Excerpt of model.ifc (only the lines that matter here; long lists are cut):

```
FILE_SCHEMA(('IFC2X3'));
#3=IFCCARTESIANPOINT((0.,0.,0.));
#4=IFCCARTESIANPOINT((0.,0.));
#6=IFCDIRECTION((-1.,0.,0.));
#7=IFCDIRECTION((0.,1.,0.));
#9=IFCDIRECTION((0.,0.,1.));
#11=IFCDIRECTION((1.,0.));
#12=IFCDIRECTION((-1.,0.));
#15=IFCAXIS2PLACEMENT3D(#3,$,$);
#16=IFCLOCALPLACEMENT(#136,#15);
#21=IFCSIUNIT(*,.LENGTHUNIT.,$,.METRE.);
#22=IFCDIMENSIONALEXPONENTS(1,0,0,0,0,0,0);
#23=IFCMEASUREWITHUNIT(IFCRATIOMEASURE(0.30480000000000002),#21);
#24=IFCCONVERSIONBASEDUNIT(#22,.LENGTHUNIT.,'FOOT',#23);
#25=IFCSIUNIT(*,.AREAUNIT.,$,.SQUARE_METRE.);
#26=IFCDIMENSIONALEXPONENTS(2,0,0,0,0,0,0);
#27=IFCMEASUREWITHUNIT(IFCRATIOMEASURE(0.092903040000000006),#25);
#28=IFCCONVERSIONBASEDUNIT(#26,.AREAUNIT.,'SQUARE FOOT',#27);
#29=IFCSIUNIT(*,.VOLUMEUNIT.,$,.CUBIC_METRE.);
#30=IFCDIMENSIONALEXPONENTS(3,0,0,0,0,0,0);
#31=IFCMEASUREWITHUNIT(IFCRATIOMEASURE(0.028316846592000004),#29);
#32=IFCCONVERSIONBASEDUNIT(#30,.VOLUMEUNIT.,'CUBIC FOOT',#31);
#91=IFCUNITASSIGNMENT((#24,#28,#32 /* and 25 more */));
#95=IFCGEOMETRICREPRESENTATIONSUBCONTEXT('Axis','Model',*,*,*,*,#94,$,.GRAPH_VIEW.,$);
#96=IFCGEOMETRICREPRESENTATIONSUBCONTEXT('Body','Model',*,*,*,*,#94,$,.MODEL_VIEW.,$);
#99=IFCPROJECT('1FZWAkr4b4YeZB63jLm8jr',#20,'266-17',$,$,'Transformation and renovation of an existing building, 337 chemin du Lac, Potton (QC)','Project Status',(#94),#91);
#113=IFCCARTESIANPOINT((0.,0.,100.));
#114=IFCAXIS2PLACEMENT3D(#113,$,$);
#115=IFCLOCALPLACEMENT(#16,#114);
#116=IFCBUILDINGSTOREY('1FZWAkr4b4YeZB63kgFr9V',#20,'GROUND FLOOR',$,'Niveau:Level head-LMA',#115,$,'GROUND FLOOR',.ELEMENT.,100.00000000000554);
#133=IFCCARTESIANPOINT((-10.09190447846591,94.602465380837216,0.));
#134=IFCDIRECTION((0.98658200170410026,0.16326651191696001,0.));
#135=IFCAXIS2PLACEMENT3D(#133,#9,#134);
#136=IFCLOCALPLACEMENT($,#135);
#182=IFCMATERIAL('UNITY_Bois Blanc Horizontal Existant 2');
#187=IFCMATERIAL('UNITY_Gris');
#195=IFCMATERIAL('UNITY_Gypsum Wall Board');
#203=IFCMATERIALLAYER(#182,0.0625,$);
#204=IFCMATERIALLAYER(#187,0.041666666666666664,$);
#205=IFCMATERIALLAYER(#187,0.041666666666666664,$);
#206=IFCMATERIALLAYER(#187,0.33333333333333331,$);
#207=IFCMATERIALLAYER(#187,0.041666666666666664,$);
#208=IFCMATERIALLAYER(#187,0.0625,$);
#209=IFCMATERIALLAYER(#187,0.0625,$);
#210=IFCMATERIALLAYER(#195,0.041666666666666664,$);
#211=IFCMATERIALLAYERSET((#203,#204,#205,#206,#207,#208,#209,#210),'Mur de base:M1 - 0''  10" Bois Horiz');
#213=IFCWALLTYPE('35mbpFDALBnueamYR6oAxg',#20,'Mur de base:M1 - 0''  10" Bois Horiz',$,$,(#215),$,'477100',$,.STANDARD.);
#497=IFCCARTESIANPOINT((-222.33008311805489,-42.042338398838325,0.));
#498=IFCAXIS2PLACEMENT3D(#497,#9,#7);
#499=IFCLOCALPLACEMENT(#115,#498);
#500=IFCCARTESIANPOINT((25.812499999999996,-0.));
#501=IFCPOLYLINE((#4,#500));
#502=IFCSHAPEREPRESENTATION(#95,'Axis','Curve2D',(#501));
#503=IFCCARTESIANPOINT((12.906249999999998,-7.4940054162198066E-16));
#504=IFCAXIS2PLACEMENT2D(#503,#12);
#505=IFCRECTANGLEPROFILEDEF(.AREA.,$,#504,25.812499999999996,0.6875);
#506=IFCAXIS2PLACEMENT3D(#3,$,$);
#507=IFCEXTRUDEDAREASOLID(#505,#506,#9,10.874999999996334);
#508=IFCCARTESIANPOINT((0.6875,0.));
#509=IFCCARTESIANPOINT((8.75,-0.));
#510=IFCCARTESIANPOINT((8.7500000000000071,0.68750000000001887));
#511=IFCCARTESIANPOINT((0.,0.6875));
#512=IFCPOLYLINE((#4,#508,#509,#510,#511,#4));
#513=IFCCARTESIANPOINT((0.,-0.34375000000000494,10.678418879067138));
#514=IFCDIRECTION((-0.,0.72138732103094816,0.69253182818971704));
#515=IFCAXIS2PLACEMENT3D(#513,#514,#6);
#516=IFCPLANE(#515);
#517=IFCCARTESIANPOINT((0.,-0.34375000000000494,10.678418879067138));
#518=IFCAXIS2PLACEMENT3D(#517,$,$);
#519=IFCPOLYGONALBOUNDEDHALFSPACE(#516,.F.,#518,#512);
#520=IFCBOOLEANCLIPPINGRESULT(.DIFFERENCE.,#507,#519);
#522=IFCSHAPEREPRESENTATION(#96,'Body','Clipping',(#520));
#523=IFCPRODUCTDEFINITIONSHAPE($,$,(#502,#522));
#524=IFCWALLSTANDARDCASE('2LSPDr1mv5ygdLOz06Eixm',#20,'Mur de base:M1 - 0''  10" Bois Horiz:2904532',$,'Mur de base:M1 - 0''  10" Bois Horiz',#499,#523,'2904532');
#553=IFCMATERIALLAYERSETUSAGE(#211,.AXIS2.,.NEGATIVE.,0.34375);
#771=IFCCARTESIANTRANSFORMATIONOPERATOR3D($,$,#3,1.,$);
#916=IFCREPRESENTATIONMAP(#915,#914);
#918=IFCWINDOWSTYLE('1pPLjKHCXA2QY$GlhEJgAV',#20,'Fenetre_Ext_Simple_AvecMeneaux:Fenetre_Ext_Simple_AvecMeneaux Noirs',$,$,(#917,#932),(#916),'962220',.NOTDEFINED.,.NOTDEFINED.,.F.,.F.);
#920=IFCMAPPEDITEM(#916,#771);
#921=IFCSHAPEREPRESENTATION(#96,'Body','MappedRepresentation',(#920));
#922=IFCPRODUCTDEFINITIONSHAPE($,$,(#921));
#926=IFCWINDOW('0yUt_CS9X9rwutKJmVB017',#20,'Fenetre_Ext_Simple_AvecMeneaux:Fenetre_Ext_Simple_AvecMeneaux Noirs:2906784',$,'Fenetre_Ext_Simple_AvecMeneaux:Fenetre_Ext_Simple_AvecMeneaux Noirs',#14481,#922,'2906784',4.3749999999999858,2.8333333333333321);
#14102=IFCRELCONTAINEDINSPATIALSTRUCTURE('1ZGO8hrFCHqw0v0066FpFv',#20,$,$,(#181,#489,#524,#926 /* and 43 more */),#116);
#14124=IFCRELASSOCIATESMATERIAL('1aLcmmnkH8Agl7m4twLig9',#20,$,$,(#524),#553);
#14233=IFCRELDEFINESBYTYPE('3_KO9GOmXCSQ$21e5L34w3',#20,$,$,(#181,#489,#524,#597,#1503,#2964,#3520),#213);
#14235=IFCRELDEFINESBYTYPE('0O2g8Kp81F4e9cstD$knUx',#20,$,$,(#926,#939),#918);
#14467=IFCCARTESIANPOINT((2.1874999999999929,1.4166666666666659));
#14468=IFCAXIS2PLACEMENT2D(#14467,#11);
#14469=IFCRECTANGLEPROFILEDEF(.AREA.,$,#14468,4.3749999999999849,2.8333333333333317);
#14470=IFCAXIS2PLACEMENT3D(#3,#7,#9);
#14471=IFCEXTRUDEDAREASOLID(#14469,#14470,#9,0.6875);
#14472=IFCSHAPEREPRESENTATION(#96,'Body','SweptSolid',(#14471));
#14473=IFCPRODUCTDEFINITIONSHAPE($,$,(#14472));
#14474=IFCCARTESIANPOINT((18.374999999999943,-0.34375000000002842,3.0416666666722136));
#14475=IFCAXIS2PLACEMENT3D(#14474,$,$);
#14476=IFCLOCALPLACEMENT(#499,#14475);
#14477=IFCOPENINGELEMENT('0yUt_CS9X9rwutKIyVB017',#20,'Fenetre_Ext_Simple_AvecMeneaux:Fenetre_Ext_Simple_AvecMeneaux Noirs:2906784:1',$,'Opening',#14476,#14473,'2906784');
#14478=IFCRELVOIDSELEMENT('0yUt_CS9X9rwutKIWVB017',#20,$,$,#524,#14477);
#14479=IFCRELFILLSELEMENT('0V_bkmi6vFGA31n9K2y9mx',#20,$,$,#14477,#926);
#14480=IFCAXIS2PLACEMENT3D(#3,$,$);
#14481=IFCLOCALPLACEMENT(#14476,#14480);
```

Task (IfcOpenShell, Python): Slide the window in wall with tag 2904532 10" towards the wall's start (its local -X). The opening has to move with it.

```python
import ifcopenshell
import ifcopenshell.api.geometry
import ifcopenshell.util.placement
import ifcopenshell.util.unit

model = ifcopenshell.open("model.ifc")
unit_scale = ifcopenshell.util.unit.calculate_unit_scale(model)

window = model.by_guid("0yUt_CS9X9rwutKJmVB017")
opening = window.FillsVoids[0].RelatingOpeningElement
wall = opening.VoidsElements[0].RelatingBuildingElement

wall_matrix = ifcopenshell.util.placement.get_local_placement(wall.ObjectPlacement)
shift = wall_matrix[:3, 0] * -10 * 0.0254 / unit_scale
before = ifcopenshell.util.placement.get_local_placement(window.ObjectPlacement)[:3, 3].copy()

# The window is placed relative to its opening, so it follows when the opening moves.
matrix = ifcopenshell.util.placement.get_local_placement(opening.ObjectPlacement)
matrix[:3, 3] += shift
ifcopenshell.api.geometry.edit_object_placement(
    model, product=opening, matrix=matrix, is_si=False, should_transform_children=True
)

after = ifcopenshell.util.placement.get_local_placement(window.ObjectPlacement)[:3, 3]
print("window moved by", (after - before).round(3) + 0.0)

model.write("model_rev.ifc")
```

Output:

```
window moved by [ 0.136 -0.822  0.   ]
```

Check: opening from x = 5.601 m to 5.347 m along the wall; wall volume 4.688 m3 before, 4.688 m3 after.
